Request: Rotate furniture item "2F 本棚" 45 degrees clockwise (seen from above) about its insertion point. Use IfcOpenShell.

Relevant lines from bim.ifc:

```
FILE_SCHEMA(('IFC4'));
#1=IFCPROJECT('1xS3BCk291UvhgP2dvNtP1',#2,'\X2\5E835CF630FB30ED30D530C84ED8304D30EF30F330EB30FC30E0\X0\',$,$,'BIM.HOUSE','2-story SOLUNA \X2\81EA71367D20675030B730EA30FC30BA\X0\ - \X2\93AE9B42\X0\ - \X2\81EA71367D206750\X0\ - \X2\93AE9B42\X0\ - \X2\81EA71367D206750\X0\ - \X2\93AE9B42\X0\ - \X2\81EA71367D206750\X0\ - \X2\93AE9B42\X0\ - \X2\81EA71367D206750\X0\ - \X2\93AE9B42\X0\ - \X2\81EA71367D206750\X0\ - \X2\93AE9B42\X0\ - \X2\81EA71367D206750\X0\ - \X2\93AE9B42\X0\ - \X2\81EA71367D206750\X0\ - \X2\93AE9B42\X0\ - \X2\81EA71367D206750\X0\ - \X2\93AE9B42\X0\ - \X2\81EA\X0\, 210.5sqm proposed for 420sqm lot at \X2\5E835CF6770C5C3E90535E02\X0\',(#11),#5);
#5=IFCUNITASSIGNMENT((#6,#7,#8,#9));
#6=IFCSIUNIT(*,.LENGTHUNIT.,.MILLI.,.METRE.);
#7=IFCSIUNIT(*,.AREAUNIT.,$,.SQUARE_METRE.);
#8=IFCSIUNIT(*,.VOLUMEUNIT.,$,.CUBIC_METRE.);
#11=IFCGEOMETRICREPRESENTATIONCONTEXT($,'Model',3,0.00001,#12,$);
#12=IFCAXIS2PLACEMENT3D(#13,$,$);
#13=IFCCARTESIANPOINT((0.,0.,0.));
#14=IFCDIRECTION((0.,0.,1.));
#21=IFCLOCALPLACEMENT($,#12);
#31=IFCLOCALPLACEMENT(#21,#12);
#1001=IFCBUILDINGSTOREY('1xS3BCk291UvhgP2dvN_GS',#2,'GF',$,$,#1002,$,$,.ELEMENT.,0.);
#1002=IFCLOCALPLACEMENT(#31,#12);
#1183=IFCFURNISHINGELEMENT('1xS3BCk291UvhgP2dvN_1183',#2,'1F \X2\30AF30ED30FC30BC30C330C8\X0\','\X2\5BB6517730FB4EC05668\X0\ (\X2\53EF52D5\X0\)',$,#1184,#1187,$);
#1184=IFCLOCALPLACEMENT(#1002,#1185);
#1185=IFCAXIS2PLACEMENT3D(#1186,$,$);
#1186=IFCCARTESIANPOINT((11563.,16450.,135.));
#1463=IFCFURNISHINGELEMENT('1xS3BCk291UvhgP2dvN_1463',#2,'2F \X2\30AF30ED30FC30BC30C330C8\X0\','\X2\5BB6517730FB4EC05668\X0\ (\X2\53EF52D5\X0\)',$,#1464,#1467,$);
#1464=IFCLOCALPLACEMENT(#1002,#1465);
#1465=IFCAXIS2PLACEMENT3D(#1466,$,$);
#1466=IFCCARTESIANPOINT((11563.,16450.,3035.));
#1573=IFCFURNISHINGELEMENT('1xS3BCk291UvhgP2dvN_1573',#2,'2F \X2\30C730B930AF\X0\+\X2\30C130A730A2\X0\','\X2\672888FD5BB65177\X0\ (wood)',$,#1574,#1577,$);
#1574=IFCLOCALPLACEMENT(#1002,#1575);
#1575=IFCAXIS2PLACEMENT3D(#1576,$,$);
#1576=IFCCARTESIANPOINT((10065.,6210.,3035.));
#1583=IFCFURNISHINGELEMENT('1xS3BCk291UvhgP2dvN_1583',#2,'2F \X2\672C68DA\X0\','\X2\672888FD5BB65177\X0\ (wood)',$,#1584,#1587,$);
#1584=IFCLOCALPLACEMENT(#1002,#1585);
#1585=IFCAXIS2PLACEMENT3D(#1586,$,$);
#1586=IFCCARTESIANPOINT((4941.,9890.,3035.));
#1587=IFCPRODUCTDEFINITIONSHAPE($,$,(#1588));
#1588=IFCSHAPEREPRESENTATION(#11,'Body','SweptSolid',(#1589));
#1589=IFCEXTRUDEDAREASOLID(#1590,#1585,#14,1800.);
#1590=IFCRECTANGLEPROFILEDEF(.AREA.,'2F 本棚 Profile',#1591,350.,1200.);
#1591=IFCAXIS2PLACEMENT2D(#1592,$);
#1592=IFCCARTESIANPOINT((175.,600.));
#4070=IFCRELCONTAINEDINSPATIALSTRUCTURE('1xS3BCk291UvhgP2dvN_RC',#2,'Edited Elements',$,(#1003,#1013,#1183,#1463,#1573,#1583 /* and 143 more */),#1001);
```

```python
import ifcopenshell
import ifcopenshell.api.geometry
import ifcopenshell.util.placement

model = ifcopenshell.open("bim.ifc")

item = model.by_id(1583)
matrix = ifcopenshell.util.placement.get_local_placement(item.ObjectPlacement)
matrix = matrix @ ifcopenshell.util.placement.rotation(-45, "Z")
ifcopenshell.api.geometry.edit_object_placement(model, product=item, matrix=matrix, is_si=False)

print(ifcopenshell.util.placement.get_local_placement(item.ObjectPlacement).round(3) + 0.0)

model.write("bim-out.ifc")
```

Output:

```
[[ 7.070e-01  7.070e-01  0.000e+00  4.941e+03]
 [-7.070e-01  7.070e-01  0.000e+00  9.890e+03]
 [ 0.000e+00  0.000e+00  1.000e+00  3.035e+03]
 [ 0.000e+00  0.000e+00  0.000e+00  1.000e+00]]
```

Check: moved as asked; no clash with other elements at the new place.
